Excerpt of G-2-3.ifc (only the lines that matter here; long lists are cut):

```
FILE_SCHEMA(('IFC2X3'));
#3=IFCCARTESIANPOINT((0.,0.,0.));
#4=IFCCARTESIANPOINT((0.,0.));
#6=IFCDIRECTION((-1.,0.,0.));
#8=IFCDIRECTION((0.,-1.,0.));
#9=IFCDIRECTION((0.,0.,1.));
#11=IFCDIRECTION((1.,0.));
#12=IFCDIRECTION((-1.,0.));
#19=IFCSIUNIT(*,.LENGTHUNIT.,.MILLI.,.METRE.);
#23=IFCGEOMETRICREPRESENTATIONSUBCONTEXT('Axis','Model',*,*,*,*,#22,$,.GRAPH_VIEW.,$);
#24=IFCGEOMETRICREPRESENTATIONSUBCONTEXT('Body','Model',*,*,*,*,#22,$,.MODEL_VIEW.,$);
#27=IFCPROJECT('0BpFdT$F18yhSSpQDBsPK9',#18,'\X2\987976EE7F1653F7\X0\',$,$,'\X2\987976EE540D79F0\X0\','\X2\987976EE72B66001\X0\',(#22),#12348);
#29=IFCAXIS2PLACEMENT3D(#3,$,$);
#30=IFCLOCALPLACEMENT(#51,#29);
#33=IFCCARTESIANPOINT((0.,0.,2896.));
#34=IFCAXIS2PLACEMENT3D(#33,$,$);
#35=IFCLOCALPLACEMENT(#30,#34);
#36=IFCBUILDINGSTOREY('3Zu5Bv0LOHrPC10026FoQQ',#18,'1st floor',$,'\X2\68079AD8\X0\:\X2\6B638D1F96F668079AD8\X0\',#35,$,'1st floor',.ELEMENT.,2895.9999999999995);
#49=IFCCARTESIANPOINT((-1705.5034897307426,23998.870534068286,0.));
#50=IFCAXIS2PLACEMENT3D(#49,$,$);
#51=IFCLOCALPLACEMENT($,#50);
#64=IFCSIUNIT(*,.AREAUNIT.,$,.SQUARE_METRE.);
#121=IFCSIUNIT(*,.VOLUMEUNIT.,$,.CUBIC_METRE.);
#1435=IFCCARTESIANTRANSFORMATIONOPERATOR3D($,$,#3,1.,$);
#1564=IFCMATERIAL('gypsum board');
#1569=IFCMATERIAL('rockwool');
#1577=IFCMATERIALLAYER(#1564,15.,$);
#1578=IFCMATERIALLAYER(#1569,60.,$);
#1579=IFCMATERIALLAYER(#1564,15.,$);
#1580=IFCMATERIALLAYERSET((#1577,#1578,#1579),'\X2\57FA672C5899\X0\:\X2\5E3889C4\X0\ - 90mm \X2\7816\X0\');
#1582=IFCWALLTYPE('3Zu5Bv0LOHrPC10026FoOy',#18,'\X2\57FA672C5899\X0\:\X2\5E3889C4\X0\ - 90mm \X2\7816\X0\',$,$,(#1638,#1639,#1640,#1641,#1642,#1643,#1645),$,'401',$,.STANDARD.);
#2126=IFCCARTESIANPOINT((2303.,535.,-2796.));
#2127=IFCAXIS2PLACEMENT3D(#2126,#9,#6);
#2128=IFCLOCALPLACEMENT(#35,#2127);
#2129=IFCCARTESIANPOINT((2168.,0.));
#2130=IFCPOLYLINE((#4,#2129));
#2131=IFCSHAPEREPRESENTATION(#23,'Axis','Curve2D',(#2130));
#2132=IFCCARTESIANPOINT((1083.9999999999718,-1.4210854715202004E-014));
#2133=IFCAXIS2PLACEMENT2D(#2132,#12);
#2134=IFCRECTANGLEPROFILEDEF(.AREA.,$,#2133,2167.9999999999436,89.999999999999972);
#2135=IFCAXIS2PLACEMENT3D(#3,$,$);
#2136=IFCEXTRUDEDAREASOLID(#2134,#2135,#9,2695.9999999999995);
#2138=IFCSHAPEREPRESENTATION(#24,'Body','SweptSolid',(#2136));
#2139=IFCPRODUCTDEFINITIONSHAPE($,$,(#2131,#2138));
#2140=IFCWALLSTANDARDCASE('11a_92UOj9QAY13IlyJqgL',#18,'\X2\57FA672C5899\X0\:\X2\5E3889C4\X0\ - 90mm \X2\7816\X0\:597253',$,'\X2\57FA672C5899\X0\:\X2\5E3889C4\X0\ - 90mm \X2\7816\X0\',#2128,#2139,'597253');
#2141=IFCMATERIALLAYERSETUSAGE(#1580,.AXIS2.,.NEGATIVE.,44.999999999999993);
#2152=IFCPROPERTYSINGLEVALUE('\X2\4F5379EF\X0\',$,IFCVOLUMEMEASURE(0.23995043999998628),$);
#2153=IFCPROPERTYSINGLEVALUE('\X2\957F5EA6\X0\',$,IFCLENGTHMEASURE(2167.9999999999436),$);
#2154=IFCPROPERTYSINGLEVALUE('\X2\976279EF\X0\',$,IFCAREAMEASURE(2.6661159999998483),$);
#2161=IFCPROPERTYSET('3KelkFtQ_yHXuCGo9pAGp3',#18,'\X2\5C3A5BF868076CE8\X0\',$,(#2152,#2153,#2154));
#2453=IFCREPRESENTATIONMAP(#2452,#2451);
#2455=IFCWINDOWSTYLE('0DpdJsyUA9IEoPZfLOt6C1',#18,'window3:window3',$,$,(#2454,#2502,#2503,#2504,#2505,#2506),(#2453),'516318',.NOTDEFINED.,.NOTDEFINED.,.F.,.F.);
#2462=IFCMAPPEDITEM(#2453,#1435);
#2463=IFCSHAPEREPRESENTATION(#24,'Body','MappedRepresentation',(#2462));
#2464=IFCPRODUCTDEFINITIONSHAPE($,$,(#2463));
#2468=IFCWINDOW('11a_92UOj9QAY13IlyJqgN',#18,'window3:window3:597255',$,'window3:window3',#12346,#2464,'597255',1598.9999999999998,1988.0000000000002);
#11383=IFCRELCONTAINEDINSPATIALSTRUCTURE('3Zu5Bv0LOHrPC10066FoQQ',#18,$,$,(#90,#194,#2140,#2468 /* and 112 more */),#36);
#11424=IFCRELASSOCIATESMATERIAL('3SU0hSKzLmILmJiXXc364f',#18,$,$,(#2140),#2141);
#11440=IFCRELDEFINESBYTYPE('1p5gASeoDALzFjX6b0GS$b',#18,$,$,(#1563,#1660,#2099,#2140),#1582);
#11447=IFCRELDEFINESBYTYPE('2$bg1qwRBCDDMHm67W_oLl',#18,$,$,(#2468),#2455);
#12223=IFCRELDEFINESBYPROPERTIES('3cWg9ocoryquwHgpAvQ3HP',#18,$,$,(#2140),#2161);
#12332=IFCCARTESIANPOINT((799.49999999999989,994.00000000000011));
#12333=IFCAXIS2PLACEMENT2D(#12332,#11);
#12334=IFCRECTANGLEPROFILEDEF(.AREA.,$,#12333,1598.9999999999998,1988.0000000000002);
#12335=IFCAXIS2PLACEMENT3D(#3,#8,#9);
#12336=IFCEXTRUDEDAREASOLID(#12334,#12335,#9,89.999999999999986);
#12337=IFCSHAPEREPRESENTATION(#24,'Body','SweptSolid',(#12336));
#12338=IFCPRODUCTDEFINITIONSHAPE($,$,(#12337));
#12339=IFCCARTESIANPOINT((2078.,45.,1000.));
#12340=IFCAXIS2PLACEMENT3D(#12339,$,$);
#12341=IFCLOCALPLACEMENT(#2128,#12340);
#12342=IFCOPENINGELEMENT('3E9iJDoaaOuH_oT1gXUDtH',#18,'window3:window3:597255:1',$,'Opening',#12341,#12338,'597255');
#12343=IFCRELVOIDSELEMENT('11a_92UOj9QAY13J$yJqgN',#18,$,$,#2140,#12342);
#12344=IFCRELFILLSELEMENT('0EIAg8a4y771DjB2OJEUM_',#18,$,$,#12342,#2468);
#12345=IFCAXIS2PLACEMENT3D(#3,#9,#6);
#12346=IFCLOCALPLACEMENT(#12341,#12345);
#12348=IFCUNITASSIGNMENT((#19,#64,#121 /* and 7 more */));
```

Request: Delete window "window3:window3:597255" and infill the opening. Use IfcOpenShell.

```python
import ifcopenshell
import ifcopenshell.api.feature
import ifcopenshell.api.pset
import ifcopenshell.api.root
import ifcopenshell.geom
import ifcopenshell.util.element
import ifcopenshell.util.shape
import ifcopenshell.util.unit

model = ifcopenshell.open("G-2-3.ifc")
area_scale = ifcopenshell.util.unit.calculate_unit_scale(model, "AREAUNIT")
volume_scale = ifcopenshell.util.unit.calculate_unit_scale(model, "VOLUMEUNIT")
settings = ifcopenshell.geom.settings()


def volume(element):
    """Net volume in cubic metres, openings subtracted."""
    shape = ifcopenshell.geom.create_shape(settings, element)
    return ifcopenshell.util.shape.get_volume(shape.geometry)


window = model.by_guid("11a_92UOj9QAY13IlyJqgN")
opening = window.FillsVoids[0].RelatingOpeningElement
wall = opening.VoidsElements[0].RelatingBuildingElement
before = volume(wall)

ifcopenshell.api.root.remove_product(model, product=window)
ifcopenshell.api.feature.remove_feature(model, feature=opening)

after = volume(wall)
thickness = 0.09  # wall thickness in metres

# Update the wall's stored quantities.
pset = model.by_id(ifcopenshell.util.element.get_pset(wall, "尺寸标注", should_inherit=False)["id"])
ifcopenshell.api.pset.edit_pset(model, pset=pset, properties={
    "体积": model.create_entity("IfcVolumeMeasure", after / volume_scale),
    "面积": model.create_entity("IfcAreaMeasure", after / thickness / area_scale),
})

print(f"wall volume {before:.3f} -> {after:.3f} m3")

model.write("G-2-3_edited.ifc")
```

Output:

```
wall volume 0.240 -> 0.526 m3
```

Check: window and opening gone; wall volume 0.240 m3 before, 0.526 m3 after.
